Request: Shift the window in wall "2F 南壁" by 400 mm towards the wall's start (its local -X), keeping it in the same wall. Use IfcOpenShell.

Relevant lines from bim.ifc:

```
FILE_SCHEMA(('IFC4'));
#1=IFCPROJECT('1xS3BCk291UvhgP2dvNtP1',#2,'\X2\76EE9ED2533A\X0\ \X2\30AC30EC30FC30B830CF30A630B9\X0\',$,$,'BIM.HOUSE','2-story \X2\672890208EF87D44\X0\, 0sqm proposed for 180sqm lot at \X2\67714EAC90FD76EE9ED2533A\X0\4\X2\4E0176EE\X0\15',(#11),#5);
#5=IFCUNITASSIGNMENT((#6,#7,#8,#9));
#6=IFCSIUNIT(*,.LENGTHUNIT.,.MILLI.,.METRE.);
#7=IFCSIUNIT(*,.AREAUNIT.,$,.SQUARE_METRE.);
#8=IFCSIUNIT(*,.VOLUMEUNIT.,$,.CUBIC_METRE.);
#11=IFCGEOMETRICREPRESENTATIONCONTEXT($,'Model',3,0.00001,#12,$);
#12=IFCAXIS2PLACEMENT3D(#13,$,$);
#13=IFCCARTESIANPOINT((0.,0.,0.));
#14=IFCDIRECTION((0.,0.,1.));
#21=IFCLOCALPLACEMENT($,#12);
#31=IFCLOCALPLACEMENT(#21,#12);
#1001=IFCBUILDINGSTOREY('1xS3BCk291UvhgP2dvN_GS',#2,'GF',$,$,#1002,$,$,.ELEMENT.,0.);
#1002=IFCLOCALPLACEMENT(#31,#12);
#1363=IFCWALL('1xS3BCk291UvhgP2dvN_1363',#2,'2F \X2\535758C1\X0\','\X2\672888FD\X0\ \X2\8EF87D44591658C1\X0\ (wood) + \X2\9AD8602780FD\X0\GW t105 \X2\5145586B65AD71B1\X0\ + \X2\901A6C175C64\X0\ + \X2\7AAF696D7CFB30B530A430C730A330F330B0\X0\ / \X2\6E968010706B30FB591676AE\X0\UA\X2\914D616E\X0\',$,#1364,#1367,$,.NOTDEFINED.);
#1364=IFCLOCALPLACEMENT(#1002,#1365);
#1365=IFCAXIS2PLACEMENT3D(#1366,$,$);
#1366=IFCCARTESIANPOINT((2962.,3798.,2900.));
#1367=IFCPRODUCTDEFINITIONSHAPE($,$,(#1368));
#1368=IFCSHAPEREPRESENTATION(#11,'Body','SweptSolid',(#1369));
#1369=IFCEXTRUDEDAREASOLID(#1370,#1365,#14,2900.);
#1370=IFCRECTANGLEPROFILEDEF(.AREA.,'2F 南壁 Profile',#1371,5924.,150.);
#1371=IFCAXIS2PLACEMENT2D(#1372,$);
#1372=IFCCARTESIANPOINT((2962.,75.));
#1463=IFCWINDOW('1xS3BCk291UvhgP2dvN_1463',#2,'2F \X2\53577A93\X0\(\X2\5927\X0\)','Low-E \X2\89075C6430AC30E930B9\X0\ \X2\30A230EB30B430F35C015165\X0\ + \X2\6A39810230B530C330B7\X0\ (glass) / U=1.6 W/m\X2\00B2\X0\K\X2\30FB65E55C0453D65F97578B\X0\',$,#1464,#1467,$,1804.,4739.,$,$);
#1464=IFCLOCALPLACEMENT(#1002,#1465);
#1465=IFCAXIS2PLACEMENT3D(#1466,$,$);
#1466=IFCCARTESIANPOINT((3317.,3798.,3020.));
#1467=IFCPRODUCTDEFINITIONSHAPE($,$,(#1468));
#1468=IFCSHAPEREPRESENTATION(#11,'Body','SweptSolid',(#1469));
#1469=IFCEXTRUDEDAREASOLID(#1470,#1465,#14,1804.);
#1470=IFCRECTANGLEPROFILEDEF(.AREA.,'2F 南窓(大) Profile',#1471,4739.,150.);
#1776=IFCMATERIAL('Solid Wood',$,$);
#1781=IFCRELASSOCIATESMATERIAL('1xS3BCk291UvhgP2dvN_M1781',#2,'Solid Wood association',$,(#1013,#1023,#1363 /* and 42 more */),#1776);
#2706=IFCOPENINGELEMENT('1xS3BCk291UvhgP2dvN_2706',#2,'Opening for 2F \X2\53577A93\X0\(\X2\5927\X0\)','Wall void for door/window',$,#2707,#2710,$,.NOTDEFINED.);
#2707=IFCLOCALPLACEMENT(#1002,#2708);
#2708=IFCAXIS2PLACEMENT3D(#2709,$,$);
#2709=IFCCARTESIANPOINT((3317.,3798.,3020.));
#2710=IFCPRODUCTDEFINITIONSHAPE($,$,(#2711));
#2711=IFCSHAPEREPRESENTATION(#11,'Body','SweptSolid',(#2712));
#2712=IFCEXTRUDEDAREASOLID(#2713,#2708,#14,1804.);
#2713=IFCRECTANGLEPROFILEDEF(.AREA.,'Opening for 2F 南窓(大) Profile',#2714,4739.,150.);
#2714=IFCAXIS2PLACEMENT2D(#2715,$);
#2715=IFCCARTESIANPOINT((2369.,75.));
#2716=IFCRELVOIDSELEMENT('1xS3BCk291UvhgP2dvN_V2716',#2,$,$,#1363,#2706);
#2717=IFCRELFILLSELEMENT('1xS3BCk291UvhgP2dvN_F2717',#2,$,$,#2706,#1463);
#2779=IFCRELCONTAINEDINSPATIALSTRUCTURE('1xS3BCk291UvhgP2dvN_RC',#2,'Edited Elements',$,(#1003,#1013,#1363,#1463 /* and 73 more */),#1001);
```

```python
import ifcopenshell
import ifcopenshell.api.geometry
import ifcopenshell.util.placement
import ifcopenshell.util.unit

model = ifcopenshell.open("bim.ifc")
unit_scale = ifcopenshell.util.unit.calculate_unit_scale(model)

window = model.by_guid("1xS3BCk291UvhgP2dvN_1463")
opening = window.FillsVoids[0].RelatingOpeningElement
wall = opening.VoidsElements[0].RelatingBuildingElement

wall_matrix = ifcopenshell.util.placement.get_local_placement(wall.ObjectPlacement)
shift = wall_matrix[:3, 0] * -0.4 / unit_scale
before = ifcopenshell.util.placement.get_local_placement(window.ObjectPlacement)[:3, 3].copy()

# The window is not placed relative to its opening, so move both.
for product in (opening, window):
    matrix = ifcopenshell.util.placement.get_local_placement(product.ObjectPlacement)
    matrix[:3, 3] += shift
    ifcopenshell.api.geometry.edit_object_placement(model, product=product, matrix=matrix, is_si=False)

after = ifcopenshell.util.placement.get_local_placement(window.ObjectPlacement)[:3, 3]
print("window moved by", (after - before).round(3) + 0.0)

model.write("bim_edited.ifc")
```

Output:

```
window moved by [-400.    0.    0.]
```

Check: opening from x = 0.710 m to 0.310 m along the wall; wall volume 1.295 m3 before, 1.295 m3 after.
